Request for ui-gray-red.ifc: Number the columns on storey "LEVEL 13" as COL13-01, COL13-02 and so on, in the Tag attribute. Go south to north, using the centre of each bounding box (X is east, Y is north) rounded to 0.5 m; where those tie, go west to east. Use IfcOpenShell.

First a look at what the model holds.

```python
import ifcopenshell
import ifcopenshell.util.element
import ifcopenshell.util.placement

model = ifcopenshell.open("ui-gray-red.ifc")
print(model.schema)
storey = next(s for s in model.by_type("IfcBuildingStorey") if s.Name == "LEVEL 13")
columns = [e for e in ifcopenshell.util.element.get_decomposition(storey) if e.is_a("IfcColumn")]
for e in sorted(columns, key=lambda e: e.id()):
    origin = ifcopenshell.util.placement.get_local_placement(e.ObjectPlacement)[:3, 3]
    print(e.id(), e.Tag, e.Name, origin.round(2) + 0.0, sep=" | ")
```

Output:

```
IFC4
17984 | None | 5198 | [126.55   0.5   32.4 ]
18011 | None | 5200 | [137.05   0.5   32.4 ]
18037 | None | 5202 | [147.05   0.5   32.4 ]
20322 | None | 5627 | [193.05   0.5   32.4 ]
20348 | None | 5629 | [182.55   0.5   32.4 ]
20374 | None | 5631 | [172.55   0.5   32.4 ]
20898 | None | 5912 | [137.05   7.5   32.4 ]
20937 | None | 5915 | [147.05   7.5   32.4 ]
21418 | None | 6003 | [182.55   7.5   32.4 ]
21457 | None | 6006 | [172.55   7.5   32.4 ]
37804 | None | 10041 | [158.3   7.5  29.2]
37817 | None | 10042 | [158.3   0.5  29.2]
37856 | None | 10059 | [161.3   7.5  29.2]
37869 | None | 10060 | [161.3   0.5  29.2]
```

```python
import ifcopenshell
import ifcopenshell.geom
import ifcopenshell.util.element
import ifcopenshell.util.shape

model = ifcopenshell.open("ui-gray-red.ifc")
settings = ifcopenshell.geom.settings()
settings.set("use-world-coords", True)


def centre(element):
    shape = ifcopenshell.geom.create_shape(settings, element)
    return ifcopenshell.util.shape.get_bbox_centroid(shape.geometry)


storey = next(s for s in model.by_type("IfcBuildingStorey") if s.Name == "LEVEL 13")
columns = [e for e in ifcopenshell.util.element.get_decomposition(storey) if e.is_a("IfcColumn")]

# Insertion points can sit at a corner or the storey origin, so sort by the geometry (in metres).
centres = {e: centre(e) for e in columns}
columns.sort(key=lambda e: (round(centres[e][1] / 0.5), centres[e][0]))

for i, e in enumerate(columns, start=1):
    number = f"COL13-{i:02d}"
    e.Tag = number
    print(e.id(), number)

model.write("ui-gray-red_updated.ifc")
```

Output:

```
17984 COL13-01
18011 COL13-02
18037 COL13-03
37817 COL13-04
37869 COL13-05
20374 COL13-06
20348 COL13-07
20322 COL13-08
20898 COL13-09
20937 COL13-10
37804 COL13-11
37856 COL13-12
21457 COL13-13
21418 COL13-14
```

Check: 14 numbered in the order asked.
